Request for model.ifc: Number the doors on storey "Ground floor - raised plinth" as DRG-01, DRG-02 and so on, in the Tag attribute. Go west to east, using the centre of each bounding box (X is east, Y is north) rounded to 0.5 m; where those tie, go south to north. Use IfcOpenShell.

First a look at what the model holds.

```python
import ifcopenshell
import ifcopenshell.util.element
import ifcopenshell.util.placement

model = ifcopenshell.open("model.ifc")
print(model.schema)
storey = next(s for s in model.by_type("IfcBuildingStorey") if s.Name == "Ground floor - raised plinth")
doors = [e for e in ifcopenshell.util.element.get_decomposition(storey) if e.is_a("IfcDoor")]
for e in sorted(doors, key=lambda e: e.id()):
    origin = ifcopenshell.util.placement.get_local_placement(e.ObjectPlacement)[:3, 3]
    print(e.id(), e.Tag, e.Name, origin.round(2) + 0.0, sep=" | ")
```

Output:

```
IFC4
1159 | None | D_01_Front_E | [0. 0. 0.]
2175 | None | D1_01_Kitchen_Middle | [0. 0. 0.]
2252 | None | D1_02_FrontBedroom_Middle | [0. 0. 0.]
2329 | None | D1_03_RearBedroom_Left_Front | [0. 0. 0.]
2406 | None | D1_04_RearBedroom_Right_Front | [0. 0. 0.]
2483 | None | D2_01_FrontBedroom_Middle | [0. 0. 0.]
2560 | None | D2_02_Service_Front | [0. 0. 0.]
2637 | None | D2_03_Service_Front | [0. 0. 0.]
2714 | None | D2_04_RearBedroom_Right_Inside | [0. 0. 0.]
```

```python
import ifcopenshell
import ifcopenshell.geom
import ifcopenshell.util.element
import ifcopenshell.util.shape

model = ifcopenshell.open("model.ifc")
settings = ifcopenshell.geom.settings()
settings.set("use-world-coords", True)


def centre(element):
    shape = ifcopenshell.geom.create_shape(settings, element)
    return ifcopenshell.util.shape.get_bbox_centroid(shape.geometry)


storey = next(s for s in model.by_type("IfcBuildingStorey") if s.Name == "Ground floor - raised plinth")
doors = [e for e in ifcopenshell.util.element.get_decomposition(storey) if e.is_a("IfcDoor")]

# Insertion points can sit at a corner or the storey origin, so sort by the geometry (in metres).
centres = {e: centre(e) for e in doors}
doors.sort(key=lambda e: (round(centres[e][0] / 0.5), centres[e][1]))

for i, e in enumerate(doors, start=1):
    number = f"DRG-{i:02d}"
    e.Tag = number
    print(e.id(), number)

model.write("model_rev.ifc")
```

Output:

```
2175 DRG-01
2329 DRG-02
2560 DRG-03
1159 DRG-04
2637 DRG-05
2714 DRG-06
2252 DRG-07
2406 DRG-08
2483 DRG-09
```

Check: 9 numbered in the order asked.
